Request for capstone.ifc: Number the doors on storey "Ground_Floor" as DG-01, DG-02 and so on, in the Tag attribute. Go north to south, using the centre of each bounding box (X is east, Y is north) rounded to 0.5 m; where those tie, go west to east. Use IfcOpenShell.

First a look at what the model holds.

```python
import ifcopenshell
import ifcopenshell.util.element
import ifcopenshell.util.placement

model = ifcopenshell.open("capstone.ifc")
print(model.schema)
storey = next(s for s in model.by_type("IfcBuildingStorey") if s.Name == "Ground_Floor")
doors = [e for e in ifcopenshell.util.element.get_decomposition(storey) if e.is_a("IfcDoor")]
for e in sorted(doors, key=lambda e: e.id()):
    origin = ifcopenshell.util.placement.get_local_placement(e.ObjectPlacement)[:3, 3]
    print(e.id(), e.Tag, e.Name, origin.round(2) + 0.0, sep=" | ")
```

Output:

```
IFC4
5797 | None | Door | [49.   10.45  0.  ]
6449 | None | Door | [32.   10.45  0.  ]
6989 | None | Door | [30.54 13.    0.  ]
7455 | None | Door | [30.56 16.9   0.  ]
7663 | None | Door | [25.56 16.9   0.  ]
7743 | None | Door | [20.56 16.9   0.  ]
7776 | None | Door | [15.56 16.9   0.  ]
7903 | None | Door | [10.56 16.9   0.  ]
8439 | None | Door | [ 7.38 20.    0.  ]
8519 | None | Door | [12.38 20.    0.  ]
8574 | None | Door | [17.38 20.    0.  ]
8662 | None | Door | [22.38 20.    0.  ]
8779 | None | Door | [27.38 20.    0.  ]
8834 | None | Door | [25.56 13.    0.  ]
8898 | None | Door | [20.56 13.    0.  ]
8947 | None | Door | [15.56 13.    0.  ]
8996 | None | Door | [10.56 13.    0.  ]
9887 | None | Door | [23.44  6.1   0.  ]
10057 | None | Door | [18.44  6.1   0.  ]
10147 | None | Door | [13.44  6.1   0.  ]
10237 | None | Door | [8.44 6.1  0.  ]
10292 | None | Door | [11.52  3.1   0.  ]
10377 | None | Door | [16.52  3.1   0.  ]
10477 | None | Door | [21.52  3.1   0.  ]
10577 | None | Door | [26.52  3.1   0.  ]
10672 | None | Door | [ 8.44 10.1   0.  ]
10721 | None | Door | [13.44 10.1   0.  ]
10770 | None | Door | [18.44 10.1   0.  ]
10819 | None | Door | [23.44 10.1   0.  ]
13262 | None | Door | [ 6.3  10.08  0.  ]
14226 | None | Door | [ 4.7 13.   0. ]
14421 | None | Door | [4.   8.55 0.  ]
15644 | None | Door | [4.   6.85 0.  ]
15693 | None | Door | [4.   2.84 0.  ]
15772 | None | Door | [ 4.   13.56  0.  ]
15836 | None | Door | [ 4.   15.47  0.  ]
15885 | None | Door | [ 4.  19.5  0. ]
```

```python
import ifcopenshell
import ifcopenshell.geom
import ifcopenshell.util.element
import ifcopenshell.util.shape

model = ifcopenshell.open("capstone.ifc")
settings = ifcopenshell.geom.settings()
settings.set("use-world-coords", True)


def centre(element):
    shape = ifcopenshell.geom.create_shape(settings, element)
    return ifcopenshell.util.shape.get_bbox_centroid(shape.geometry)


storey = next(s for s in model.by_type("IfcBuildingStorey") if s.Name == "Ground_Floor")
doors = [e for e in ifcopenshell.util.element.get_decomposition(storey) if e.is_a("IfcDoor")]

# Insertion points can sit at a corner or the storey origin, so sort by the geometry (in metres).
centres = {e: centre(e) for e in doors}
doors.sort(key=lambda e: (-round(centres[e][1] / 0.5), centres[e][0]))

for i, e in enumerate(doors, start=1):
    number = f"DG-{i:02d}"
    e.Tag = number
    print(e.id(), number)

model.write("capstone_edited.ifc")
```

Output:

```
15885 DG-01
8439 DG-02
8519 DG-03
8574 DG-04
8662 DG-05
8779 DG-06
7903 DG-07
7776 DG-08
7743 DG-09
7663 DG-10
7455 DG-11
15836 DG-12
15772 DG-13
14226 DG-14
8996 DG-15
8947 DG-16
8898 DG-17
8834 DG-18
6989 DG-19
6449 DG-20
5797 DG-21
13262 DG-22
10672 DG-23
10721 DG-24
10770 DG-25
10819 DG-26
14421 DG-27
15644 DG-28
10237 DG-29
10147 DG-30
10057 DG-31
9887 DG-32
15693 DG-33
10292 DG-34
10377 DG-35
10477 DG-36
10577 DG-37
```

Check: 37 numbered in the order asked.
